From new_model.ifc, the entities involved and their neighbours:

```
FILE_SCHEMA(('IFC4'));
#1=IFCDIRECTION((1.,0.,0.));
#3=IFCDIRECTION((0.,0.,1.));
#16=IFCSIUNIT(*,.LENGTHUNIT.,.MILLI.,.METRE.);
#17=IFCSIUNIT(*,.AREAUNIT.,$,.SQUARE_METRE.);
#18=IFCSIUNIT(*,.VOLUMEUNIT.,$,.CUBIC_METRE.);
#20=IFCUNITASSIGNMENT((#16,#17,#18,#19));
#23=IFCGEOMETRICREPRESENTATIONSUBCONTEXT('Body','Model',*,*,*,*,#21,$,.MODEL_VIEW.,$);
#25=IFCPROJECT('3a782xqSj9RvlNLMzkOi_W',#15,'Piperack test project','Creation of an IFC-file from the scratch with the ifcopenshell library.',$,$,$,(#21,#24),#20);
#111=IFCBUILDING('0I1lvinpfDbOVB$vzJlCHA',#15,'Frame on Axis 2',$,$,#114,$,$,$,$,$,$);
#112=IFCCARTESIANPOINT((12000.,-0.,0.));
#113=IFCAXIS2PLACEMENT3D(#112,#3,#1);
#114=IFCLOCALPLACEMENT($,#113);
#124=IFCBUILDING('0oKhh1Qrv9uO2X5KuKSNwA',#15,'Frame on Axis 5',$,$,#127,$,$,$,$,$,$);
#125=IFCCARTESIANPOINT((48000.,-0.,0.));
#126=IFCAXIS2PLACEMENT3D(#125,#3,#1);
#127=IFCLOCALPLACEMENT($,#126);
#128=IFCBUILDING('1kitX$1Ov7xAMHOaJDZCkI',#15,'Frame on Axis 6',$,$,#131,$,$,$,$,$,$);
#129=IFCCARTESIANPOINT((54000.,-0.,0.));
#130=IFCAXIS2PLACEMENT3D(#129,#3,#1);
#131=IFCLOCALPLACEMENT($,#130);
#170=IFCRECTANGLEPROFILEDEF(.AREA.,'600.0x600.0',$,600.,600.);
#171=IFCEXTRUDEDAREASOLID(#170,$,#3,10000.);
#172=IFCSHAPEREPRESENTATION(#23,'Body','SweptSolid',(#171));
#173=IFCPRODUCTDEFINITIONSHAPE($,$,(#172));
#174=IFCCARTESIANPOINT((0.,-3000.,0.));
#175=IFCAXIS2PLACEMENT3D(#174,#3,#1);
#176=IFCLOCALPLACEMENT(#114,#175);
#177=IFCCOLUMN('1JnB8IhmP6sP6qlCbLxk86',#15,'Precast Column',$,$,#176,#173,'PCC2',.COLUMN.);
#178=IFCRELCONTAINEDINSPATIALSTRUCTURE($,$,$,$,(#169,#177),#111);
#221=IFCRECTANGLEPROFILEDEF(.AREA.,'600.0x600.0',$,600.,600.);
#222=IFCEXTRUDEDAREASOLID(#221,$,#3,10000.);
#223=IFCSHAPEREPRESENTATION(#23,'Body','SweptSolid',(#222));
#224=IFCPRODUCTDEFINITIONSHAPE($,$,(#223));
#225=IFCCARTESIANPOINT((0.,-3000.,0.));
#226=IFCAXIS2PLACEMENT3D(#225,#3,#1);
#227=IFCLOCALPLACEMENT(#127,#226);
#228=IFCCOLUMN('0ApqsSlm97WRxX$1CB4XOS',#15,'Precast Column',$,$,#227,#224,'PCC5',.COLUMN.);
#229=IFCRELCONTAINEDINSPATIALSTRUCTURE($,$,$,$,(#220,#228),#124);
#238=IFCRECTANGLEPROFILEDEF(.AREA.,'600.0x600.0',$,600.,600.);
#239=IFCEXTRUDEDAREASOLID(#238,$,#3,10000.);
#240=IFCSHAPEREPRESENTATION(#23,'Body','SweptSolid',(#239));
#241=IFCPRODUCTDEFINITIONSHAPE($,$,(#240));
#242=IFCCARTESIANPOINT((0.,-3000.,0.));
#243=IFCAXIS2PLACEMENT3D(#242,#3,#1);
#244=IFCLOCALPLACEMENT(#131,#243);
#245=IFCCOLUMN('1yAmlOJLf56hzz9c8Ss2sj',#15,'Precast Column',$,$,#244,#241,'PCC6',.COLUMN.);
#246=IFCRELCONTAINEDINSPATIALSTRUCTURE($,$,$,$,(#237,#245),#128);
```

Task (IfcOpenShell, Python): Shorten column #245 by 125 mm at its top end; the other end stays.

```python
import ifcopenshell
import ifcopenshell.util.representation
import ifcopenshell.util.unit

model = ifcopenshell.open("new_model.ifc")
unit_scale = ifcopenshell.util.unit.calculate_unit_scale(model)

member = model.by_guid("1yAmlOJLf56hzz9c8Ss2sj")
change = -0.125 / unit_scale

# The extrusion runs towards the end named, so only its depth changes.
body = ifcopenshell.util.representation.get_representation(member, "Model", "Body")
solid = body.Items[0]
old_length = solid.Depth
solid.Depth += change

print(f"length {old_length:g} -> {solid.Depth:g}")

model.write("new_model_rev.ifc")
```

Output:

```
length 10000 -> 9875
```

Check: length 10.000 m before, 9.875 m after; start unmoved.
